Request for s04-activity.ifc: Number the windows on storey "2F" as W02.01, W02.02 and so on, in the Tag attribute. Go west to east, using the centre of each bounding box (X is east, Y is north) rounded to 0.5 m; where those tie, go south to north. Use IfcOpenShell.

First a look at what the model holds.

```python
import ifcopenshell
import ifcopenshell.util.element
import ifcopenshell.util.placement

model = ifcopenshell.open("s04-activity.ifc")
print(model.schema)
storey = next(s for s in model.by_type("IfcBuildingStorey") if s.Name == "2F")
windows = [e for e in ifcopenshell.util.element.get_decomposition(storey) if e.is_a("IfcWindow")]
for e in sorted(windows, key=lambda e: e.id()):
    origin = ifcopenshell.util.placement.get_local_placement(e.ObjectPlacement)[:3, 3]
    print(e.id(), e.Tag, e.Name, origin.round(2) + 0.0, sep=" | ")
```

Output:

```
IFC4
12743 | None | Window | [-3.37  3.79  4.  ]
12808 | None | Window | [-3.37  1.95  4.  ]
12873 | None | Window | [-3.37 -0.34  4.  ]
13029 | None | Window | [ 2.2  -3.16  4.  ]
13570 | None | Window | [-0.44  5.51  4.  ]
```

```python
import ifcopenshell
import ifcopenshell.geom
import ifcopenshell.util.element
import ifcopenshell.util.shape

model = ifcopenshell.open("s04-activity.ifc")
settings = ifcopenshell.geom.settings()
settings.set("use-world-coords", True)


def centre(element):
    shape = ifcopenshell.geom.create_shape(settings, element)
    return ifcopenshell.util.shape.get_bbox_centroid(shape.geometry)


storey = next(s for s in model.by_type("IfcBuildingStorey") if s.Name == "2F")
windows = [e for e in ifcopenshell.util.element.get_decomposition(storey) if e.is_a("IfcWindow")]

# Insertion points can sit at a corner or the storey origin, so sort by the geometry (in metres).
centres = {e: centre(e) for e in windows}
windows.sort(key=lambda e: (round(centres[e][0] / 0.5), centres[e][1]))

for i, e in enumerate(windows, start=1):
    number = f"W02.{i:02d}"
    e.Tag = number
    print(e.id(), number)

model.write("s04-activity_rev.ifc")
```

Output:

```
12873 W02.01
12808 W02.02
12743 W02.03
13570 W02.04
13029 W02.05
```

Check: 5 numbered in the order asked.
